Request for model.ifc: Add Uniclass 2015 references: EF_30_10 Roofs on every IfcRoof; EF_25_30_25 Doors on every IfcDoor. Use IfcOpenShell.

First a look at what the model holds.

```python
import ifcopenshell

model = ifcopenshell.open("model.ifc")
print(model.schema)
print("classifications:", [c.Name for c in model.by_type("IfcClassification")])
for ifc_class in ("IfcDoor", "IfcRoof", "IfcStair", "IfcWall", "IfcWindow"):
    print(ifc_class, len(model.by_type(ifc_class)))
```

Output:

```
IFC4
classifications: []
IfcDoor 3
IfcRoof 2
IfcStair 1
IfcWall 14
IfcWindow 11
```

```python
import ifcopenshell
import ifcopenshell.api.classification

model = ifcopenshell.open("model.ifc")

system = ifcopenshell.api.classification.add_classification(model, classification="Uniclass 2015")

codes = {
    "IfcRoof": ("EF_30_10", "Roofs"),
    "IfcDoor": ("EF_25_30_25", "Doors"),
}
for ifc_class, (code, name) in codes.items():
    products = model.by_type(ifc_class)
    ifcopenshell.api.classification.add_reference(
        model, products=products, classification=system, identification=code, name=name
    )
    print(code, len(products))

model.write("model_v2.ifc")
```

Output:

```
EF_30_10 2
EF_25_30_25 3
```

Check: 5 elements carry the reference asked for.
